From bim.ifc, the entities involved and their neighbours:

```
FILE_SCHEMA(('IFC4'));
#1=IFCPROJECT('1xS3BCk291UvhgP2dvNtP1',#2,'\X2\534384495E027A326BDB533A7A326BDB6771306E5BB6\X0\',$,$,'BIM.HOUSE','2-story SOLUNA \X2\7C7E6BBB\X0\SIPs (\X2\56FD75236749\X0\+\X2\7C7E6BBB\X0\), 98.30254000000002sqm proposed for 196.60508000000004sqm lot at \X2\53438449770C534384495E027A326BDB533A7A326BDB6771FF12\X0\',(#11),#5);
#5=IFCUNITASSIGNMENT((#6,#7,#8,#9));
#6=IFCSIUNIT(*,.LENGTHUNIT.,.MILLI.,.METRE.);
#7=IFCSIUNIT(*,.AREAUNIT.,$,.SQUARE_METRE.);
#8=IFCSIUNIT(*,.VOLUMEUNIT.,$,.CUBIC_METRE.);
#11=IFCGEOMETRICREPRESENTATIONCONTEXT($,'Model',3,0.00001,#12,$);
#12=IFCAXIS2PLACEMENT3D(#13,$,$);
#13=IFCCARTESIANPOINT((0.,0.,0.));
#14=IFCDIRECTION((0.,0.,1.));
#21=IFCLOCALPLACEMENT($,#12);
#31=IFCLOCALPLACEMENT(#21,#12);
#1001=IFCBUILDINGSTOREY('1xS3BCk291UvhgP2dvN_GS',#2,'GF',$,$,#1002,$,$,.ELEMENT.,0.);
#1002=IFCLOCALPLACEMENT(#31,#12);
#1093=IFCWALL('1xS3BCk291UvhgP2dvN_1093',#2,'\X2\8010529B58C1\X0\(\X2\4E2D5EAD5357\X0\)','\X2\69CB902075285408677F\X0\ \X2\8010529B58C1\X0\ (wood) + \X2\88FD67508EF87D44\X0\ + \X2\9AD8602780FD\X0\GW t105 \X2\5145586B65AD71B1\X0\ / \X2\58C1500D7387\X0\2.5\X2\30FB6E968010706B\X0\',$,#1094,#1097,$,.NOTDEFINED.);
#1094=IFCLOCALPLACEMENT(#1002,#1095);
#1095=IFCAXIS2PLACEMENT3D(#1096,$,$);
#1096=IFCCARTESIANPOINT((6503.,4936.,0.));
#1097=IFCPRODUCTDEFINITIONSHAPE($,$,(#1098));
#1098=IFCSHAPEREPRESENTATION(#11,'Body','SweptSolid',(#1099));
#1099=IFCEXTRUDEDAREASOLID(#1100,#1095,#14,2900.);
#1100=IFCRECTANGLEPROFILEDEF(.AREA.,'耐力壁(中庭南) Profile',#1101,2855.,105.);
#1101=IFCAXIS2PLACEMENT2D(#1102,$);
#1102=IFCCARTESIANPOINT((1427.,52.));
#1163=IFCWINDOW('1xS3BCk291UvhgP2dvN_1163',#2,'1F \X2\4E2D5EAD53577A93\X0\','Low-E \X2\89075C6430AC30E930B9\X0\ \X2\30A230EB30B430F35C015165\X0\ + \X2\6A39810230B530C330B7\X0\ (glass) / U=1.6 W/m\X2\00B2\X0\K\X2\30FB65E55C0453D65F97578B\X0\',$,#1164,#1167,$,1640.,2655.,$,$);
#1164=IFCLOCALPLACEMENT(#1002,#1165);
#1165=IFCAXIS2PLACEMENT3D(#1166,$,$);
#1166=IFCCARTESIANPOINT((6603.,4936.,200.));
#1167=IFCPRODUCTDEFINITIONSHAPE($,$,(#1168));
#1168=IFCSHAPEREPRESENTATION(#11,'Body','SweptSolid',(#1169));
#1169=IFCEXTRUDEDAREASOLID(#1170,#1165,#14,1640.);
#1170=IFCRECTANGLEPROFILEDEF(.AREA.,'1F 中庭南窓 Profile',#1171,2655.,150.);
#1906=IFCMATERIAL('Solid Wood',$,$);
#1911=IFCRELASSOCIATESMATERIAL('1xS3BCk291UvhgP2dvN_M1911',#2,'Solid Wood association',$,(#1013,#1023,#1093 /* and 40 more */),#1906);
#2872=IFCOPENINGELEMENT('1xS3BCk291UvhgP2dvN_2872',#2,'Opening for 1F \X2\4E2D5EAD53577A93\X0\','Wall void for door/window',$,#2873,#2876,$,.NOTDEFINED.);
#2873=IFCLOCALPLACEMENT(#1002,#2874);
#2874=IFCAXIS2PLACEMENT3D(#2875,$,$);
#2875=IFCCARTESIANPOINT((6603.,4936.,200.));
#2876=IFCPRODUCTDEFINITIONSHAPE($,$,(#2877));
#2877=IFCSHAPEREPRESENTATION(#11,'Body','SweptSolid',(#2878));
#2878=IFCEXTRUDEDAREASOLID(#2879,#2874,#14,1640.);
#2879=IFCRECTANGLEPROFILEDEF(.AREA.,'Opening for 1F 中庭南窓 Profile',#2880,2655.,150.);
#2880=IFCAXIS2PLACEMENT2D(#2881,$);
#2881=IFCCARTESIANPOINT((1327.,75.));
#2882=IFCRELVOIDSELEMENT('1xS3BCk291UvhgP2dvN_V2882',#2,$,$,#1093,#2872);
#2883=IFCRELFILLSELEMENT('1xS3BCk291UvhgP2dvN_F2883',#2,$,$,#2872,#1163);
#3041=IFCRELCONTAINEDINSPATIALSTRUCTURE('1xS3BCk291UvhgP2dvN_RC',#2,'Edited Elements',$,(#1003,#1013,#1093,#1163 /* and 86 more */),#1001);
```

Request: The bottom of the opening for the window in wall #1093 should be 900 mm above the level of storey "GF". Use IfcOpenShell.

```python
import numpy as np
import ifcopenshell
import ifcopenshell.api.geometry
import ifcopenshell.geom
import ifcopenshell.util.element
import ifcopenshell.util.placement
import ifcopenshell.util.shape
import ifcopenshell.util.unit

model = ifcopenshell.open("bim.ifc")
unit_scale = ifcopenshell.util.unit.calculate_unit_scale(model)

window = model.by_guid("1xS3BCk291UvhgP2dvN_1163")
opening = window.FillsVoids[0].RelatingOpeningElement
storey = ifcopenshell.util.element.get_container(window, ifc_class="IfcBuildingStorey")
level = ifcopenshell.util.placement.get_local_placement(storey.ObjectPlacement)[2, 3]

# The opening's origin need not be at the sill, so measure its lowest point.
shape = ifcopenshell.geom.create_shape(ifcopenshell.geom.settings(), opening)
bottom = ifcopenshell.util.shape.get_shape_bottom_elevation(shape, shape.geometry) / unit_scale
dz = level + 0.9 / unit_scale - bottom

shift = np.array([0.0, 0.0, dz])
# The window is not placed relative to its opening, so move both.
for product in (opening, window):
    matrix = ifcopenshell.util.placement.get_local_placement(product.ObjectPlacement)
    matrix[:3, 3] += shift
    ifcopenshell.api.geometry.edit_object_placement(model, product=product, matrix=matrix, is_si=False)

print(f"moved by {dz * unit_scale:+.3f} m")

model.write("bim_rev.ifc")
```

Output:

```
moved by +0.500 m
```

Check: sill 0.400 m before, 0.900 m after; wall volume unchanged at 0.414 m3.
